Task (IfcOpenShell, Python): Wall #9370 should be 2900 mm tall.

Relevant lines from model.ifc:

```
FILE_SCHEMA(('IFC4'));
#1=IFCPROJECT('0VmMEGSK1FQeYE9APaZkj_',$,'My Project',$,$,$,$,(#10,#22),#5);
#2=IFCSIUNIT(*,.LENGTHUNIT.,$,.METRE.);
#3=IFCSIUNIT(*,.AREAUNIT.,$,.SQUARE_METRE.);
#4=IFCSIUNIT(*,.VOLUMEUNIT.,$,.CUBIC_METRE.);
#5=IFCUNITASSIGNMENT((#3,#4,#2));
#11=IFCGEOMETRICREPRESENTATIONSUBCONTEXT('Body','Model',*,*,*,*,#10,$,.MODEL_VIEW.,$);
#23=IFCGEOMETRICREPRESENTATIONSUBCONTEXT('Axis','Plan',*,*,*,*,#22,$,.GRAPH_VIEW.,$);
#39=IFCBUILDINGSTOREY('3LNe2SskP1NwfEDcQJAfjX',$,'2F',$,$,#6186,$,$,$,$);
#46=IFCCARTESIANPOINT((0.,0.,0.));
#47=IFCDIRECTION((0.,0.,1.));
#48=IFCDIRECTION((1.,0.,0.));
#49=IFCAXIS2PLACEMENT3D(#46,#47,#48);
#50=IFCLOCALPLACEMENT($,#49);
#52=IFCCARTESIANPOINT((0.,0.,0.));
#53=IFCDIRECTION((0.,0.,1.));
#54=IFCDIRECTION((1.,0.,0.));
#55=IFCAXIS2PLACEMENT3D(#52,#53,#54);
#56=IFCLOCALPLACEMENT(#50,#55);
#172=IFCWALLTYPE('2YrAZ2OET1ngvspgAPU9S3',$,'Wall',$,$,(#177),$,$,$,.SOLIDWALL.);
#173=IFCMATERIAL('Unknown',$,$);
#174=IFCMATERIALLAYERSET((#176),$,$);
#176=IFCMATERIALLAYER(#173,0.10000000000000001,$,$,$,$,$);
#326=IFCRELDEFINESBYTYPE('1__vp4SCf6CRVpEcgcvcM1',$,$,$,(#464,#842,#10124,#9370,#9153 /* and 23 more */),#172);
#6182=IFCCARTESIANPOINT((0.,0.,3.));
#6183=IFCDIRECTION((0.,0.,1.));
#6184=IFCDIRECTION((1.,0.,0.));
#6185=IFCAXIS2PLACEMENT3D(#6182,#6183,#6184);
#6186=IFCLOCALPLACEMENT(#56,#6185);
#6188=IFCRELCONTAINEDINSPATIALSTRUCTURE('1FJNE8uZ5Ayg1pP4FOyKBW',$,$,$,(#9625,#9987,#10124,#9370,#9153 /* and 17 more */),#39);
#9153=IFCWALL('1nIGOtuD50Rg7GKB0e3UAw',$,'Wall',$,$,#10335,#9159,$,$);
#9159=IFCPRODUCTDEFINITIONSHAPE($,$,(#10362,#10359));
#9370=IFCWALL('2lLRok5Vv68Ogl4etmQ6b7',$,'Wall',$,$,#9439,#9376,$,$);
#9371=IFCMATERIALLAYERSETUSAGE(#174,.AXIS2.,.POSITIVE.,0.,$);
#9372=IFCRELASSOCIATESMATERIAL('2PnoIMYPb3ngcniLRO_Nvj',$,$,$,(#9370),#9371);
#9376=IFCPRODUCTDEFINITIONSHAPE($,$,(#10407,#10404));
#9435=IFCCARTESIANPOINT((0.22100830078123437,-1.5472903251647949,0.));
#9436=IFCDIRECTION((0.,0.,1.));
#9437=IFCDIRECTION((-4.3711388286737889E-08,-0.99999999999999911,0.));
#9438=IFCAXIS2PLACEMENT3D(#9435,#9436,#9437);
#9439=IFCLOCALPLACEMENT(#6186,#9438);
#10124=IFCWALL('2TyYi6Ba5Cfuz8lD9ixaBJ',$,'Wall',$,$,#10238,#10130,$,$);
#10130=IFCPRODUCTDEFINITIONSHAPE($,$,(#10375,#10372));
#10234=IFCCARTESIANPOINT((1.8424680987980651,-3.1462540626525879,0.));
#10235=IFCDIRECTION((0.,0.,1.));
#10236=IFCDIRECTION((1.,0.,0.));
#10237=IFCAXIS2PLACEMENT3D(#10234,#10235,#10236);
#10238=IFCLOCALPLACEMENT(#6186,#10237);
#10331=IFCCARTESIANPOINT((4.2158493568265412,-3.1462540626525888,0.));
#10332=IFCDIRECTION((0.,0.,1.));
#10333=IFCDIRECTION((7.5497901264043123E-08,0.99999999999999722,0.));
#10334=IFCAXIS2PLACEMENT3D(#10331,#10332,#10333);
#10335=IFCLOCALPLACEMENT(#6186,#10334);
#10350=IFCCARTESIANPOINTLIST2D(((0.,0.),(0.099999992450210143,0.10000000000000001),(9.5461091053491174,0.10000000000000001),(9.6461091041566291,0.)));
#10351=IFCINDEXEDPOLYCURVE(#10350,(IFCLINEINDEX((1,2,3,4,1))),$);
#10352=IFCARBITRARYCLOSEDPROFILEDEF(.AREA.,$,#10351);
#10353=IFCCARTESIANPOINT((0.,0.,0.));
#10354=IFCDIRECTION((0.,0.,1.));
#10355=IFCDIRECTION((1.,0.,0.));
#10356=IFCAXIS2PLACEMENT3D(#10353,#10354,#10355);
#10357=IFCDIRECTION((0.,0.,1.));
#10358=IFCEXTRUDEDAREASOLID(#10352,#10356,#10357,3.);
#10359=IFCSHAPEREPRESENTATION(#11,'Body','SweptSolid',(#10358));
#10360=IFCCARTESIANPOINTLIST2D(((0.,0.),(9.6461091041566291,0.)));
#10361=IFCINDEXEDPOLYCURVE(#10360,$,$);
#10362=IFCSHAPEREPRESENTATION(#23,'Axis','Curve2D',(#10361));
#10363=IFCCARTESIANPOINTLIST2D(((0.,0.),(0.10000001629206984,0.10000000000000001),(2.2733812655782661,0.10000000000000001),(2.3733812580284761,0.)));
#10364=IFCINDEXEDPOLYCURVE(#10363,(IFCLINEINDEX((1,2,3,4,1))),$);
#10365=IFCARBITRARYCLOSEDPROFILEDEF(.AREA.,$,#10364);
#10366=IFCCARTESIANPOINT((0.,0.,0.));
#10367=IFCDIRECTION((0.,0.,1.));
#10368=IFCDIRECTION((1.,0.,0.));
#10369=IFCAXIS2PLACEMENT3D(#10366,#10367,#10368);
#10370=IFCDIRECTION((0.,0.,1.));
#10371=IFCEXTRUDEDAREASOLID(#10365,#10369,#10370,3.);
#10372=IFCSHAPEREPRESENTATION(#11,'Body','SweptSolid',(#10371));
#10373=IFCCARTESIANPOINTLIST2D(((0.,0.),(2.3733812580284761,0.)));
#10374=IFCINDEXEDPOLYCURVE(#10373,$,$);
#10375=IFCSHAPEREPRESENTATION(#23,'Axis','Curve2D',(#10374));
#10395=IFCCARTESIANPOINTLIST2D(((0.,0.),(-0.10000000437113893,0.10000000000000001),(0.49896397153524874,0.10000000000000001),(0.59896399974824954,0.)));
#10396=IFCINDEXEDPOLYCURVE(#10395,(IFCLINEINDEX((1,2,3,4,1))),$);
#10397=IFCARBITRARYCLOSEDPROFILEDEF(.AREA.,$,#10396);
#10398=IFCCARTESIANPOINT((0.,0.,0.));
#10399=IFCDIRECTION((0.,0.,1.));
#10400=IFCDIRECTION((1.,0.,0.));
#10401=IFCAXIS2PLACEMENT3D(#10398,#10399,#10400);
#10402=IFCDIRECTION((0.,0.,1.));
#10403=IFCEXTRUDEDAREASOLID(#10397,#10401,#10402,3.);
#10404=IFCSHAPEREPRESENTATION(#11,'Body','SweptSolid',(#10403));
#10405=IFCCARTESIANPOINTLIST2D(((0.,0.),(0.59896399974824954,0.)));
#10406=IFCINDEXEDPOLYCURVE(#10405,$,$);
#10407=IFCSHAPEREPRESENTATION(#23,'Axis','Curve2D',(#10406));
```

```python
import ifcopenshell
import ifcopenshell.geom
import ifcopenshell.util.representation
import ifcopenshell.util.shape

model = ifcopenshell.open("model.ifc")
settings = ifcopenshell.geom.settings()


def volume(element):
    """Net volume in cubic metres, openings subtracted."""
    shape = ifcopenshell.geom.create_shape(settings, element)
    return ifcopenshell.util.shape.get_volume(shape.geometry)


wall = model.by_guid("2lLRok5Vv68Ogl4etmQ6b7")
before = volume(wall)

body = ifcopenshell.util.representation.get_representation(wall, "Model", "Body")
solid = body.Items[0]
old_height = solid.Depth
solid.Depth = 2.9
after = volume(wall)

print(f"height {old_height:g} -> {solid.Depth:g}, volume {before:.3f} -> {after:.3f} m3")

model.write("model_v2.ifc")
```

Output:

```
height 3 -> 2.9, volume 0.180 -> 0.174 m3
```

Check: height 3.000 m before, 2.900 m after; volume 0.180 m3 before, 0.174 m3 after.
